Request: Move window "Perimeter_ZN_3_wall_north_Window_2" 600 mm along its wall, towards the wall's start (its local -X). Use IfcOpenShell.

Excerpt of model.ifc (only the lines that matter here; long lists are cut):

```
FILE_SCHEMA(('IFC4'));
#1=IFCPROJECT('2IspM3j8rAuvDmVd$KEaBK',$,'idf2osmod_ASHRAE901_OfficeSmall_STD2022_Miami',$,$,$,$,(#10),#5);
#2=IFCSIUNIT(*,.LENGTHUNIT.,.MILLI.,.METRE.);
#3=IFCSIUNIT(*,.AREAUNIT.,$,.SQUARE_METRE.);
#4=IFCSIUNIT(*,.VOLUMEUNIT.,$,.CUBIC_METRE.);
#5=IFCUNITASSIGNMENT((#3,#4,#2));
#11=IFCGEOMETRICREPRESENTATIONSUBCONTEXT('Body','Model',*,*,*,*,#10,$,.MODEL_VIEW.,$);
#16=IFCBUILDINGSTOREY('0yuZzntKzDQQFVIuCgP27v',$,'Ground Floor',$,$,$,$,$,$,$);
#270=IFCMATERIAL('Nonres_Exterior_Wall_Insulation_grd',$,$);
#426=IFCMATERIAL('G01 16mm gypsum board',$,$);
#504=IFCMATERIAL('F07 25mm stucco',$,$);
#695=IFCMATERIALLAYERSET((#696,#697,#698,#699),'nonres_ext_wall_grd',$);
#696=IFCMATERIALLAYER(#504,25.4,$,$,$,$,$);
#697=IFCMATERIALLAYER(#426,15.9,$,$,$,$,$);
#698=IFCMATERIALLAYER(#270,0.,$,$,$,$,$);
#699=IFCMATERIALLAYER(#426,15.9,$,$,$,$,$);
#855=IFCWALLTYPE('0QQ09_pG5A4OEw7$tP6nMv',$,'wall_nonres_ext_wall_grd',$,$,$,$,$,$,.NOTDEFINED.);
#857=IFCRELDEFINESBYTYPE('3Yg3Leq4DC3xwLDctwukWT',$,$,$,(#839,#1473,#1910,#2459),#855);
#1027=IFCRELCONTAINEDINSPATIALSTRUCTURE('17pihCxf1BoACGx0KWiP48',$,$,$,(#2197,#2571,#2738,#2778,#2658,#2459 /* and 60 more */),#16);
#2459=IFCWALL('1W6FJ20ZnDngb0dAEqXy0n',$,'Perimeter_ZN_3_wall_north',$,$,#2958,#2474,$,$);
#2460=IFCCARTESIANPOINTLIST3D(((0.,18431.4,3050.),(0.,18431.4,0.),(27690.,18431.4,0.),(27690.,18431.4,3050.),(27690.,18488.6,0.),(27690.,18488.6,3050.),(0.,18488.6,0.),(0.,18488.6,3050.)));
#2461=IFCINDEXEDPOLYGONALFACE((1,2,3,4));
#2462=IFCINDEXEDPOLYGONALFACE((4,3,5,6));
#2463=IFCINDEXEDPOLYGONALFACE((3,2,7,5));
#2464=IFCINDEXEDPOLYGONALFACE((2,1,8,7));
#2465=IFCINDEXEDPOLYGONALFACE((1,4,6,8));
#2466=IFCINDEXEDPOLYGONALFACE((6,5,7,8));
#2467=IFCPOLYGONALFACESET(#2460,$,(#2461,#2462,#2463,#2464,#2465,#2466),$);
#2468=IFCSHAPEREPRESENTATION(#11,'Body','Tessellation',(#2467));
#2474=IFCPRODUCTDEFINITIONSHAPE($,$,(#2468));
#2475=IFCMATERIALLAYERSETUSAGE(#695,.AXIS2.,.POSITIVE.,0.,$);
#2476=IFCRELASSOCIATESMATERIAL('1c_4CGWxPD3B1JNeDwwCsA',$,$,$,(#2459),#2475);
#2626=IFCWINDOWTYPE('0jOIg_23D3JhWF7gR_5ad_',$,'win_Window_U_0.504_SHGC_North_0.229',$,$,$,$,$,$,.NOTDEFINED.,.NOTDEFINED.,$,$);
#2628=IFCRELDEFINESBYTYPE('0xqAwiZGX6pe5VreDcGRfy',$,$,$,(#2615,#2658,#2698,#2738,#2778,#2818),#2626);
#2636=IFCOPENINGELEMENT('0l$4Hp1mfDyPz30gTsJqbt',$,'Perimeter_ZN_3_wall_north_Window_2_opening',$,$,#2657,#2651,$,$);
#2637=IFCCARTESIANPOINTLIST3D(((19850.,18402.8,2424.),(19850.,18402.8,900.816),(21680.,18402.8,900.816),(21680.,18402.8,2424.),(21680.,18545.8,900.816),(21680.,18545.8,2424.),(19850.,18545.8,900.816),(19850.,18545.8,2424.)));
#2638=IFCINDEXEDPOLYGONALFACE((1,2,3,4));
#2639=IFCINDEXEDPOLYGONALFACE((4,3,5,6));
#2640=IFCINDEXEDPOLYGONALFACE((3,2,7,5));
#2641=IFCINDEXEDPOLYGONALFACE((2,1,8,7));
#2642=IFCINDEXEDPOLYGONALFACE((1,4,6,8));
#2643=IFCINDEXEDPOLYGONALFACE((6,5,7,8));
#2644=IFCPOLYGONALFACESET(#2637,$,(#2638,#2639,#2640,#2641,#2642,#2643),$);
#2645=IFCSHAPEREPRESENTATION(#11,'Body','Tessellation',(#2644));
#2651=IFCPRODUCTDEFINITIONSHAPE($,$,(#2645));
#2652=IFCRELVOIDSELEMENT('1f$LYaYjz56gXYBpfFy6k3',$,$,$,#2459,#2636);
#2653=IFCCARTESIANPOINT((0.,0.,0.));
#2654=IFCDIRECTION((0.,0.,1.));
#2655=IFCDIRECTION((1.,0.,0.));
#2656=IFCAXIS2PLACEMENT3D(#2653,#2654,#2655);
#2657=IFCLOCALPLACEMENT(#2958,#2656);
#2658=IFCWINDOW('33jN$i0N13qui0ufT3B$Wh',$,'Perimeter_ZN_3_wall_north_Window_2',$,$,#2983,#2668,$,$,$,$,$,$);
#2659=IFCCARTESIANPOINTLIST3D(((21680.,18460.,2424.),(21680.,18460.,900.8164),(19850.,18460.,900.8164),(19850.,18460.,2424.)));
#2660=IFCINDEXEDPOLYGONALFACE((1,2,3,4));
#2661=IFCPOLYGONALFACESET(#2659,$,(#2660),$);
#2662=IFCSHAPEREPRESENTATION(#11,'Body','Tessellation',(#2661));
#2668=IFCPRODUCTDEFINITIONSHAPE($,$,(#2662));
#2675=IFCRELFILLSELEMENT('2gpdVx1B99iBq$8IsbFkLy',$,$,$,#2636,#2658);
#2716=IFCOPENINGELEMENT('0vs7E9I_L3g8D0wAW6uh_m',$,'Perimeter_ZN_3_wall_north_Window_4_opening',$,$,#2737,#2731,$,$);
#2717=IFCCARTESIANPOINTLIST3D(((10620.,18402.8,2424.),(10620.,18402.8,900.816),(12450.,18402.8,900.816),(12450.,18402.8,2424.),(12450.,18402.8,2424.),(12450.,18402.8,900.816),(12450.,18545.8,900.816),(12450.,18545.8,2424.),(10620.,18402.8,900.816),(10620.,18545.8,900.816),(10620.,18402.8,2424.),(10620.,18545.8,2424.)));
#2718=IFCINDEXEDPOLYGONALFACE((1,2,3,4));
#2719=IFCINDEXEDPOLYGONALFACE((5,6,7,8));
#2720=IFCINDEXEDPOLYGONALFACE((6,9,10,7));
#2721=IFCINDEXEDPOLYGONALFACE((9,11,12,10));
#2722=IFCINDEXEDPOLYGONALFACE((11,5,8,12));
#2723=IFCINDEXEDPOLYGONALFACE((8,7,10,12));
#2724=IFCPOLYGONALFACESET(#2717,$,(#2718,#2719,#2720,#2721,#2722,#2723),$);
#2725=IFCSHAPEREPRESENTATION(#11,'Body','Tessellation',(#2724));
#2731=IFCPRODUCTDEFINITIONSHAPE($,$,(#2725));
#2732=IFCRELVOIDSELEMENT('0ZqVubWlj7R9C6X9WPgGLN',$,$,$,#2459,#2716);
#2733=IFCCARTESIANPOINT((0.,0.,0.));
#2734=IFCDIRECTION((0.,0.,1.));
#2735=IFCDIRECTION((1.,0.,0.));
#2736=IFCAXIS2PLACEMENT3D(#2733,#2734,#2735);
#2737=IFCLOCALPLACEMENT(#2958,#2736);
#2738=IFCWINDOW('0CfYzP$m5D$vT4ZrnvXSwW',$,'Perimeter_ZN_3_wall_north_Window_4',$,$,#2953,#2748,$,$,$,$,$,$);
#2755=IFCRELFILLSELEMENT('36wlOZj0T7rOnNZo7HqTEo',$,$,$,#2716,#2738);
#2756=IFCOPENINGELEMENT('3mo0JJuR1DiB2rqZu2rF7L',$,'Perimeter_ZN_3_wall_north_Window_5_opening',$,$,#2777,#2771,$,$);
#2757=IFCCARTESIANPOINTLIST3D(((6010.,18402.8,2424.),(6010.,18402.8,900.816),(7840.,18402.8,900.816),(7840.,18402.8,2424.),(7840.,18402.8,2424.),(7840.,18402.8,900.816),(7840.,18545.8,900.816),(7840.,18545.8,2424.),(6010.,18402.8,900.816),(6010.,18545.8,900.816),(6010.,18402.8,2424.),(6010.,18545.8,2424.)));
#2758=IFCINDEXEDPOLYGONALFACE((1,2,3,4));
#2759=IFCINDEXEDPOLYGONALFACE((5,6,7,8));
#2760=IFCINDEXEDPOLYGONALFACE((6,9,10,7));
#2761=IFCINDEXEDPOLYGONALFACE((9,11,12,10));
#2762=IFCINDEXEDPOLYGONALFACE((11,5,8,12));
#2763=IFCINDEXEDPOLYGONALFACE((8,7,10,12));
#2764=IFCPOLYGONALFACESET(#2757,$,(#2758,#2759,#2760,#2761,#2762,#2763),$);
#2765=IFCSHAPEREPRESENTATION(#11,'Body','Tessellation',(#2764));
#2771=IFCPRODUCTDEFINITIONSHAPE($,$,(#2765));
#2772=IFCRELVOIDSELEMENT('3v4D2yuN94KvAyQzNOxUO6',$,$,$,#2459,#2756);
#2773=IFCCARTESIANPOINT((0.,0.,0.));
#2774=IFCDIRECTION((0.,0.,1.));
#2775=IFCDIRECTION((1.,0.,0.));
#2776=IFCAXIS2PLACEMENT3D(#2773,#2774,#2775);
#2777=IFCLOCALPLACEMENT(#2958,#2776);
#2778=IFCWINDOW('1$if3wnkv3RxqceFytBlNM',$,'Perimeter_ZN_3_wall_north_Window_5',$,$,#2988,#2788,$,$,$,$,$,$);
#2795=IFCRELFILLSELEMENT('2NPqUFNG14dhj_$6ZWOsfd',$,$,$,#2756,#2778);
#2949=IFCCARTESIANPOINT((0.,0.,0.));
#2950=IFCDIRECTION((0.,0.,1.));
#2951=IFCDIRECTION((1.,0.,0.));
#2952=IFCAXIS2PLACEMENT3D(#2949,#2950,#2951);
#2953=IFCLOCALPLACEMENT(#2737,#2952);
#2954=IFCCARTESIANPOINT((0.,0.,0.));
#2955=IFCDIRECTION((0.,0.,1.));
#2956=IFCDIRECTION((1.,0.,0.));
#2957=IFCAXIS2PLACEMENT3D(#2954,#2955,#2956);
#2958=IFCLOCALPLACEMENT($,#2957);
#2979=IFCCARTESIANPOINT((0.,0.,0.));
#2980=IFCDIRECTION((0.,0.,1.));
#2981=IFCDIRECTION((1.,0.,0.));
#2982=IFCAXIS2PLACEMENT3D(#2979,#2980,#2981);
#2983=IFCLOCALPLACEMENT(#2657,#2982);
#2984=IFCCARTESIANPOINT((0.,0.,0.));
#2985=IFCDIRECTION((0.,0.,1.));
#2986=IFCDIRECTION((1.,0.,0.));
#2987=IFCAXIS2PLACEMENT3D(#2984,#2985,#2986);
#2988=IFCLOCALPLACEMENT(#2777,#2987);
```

```python
import ifcopenshell
import ifcopenshell.api.geometry
import ifcopenshell.util.placement
import ifcopenshell.util.unit

model = ifcopenshell.open("model.ifc")
unit_scale = ifcopenshell.util.unit.calculate_unit_scale(model)

window = model.by_id(2658)
opening = window.FillsVoids[0].RelatingOpeningElement
wall = opening.VoidsElements[0].RelatingBuildingElement

wall_matrix = ifcopenshell.util.placement.get_local_placement(wall.ObjectPlacement)
shift = wall_matrix[:3, 0] * -0.6 / unit_scale
before = ifcopenshell.util.placement.get_local_placement(window.ObjectPlacement)[:3, 3].copy()

# The window is placed relative to its opening, so it follows when the opening moves.
matrix = ifcopenshell.util.placement.get_local_placement(opening.ObjectPlacement)
matrix[:3, 3] += shift
ifcopenshell.api.geometry.edit_object_placement(
    model, product=opening, matrix=matrix, is_si=False, should_transform_children=True
)

after = ifcopenshell.util.placement.get_local_placement(window.ObjectPlacement)[:3, 3]
print("window moved by", (after - before).round(3) + 0.0)

model.write("model-out.ifc")
```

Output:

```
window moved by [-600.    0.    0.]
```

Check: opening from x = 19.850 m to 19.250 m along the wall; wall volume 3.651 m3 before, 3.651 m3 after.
